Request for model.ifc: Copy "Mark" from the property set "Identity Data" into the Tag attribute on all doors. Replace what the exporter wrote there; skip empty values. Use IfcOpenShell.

First a look at what the model holds.

```python
import ifcopenshell
import ifcopenshell.util.element

model = ifcopenshell.open("model.ifc")
print(model.schema)
doors = model.by_type("IfcDoor")
print(len(doors), "doors")
for e in doors[:8]:
    source = ifcopenshell.util.element.get_pset(e, "Identity Data", "Mark")
    target = e.Tag
    print(e.id(), repr(source), repr(target), sep=" | ")
```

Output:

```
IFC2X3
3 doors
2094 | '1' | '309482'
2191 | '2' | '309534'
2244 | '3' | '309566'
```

```python
import ifcopenshell
import ifcopenshell.util.element

model = ifcopenshell.open("model.ifc")

count = 0
for e in model.by_type("IfcDoor"):
    value = ifcopenshell.util.element.get_pset(e, "Identity Data", "Mark")
    current = e.Tag
    if not value or not value.strip() or current == value:
        continue
    e.Tag = value
    count += 1

print(count, "doors updated")

model.write("model_edited.ifc")
```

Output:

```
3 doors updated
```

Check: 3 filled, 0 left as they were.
